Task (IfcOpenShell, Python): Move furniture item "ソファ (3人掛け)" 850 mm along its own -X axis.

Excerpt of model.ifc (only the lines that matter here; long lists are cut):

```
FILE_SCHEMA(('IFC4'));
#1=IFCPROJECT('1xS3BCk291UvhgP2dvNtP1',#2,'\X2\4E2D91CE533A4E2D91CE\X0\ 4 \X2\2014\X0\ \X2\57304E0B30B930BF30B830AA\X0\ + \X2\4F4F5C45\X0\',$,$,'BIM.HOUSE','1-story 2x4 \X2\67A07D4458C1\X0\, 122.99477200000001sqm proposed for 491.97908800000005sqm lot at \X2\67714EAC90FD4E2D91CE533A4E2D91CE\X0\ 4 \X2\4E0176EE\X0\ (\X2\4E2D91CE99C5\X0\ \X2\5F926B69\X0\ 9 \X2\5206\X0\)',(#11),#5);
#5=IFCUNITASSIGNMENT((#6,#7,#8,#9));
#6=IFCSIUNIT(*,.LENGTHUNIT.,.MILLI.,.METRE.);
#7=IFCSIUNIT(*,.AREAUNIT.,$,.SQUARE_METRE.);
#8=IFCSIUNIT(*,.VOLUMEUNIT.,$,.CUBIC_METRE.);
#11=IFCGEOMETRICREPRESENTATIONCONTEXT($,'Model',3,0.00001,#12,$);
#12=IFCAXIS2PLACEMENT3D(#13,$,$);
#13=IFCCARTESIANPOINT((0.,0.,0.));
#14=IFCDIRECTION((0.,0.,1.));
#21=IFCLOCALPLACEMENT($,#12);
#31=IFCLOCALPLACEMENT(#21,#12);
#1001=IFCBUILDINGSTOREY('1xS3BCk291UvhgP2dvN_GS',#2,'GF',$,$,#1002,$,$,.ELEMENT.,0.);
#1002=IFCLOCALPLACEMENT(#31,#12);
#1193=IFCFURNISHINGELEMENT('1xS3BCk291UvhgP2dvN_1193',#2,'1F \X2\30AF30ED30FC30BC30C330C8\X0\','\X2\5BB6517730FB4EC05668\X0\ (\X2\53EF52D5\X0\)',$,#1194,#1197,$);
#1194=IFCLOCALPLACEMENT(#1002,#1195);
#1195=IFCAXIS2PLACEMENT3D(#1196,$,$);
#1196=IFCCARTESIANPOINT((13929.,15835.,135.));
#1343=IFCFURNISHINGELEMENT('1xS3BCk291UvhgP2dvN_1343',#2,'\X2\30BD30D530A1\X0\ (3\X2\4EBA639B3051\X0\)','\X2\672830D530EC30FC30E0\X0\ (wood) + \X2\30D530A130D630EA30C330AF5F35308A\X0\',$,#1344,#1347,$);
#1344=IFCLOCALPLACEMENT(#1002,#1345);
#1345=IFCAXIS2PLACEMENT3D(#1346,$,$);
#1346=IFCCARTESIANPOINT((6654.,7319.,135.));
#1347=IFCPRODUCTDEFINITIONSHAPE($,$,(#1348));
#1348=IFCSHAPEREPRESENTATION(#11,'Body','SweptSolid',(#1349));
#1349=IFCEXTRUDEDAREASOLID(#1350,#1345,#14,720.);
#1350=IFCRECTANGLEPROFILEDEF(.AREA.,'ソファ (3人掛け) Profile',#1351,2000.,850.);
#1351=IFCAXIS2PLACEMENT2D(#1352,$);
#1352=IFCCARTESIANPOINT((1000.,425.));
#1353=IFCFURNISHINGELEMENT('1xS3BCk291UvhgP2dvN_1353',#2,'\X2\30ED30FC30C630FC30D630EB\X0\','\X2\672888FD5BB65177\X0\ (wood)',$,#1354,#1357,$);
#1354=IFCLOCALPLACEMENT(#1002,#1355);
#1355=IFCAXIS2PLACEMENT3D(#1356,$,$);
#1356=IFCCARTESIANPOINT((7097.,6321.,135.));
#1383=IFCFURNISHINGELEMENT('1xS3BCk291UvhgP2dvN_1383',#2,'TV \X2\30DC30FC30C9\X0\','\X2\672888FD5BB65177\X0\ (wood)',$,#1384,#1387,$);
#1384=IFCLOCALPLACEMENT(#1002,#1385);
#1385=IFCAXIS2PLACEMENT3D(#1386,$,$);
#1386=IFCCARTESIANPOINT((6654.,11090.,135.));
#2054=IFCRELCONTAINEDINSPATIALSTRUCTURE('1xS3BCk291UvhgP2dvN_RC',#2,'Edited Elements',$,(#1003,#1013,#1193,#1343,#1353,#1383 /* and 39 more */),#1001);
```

```python
import ifcopenshell
import ifcopenshell.api.geometry
import ifcopenshell.util.placement

model = ifcopenshell.open("model.ifc")

item = model.by_id(1343)
matrix = ifcopenshell.util.placement.get_local_placement(item.ObjectPlacement)
matrix[:3, 3] -= matrix[:3, 0] * 850.0
ifcopenshell.api.geometry.edit_object_placement(model, product=item, matrix=matrix, is_si=False)

print(ifcopenshell.util.placement.get_local_placement(item.ObjectPlacement).round(3) + 0.0)

model.write("model_updated.ifc")
```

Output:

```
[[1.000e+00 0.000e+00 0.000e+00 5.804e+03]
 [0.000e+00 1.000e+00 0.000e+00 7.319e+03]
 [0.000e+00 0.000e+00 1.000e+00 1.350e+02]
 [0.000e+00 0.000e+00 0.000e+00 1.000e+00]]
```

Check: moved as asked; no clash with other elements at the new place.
